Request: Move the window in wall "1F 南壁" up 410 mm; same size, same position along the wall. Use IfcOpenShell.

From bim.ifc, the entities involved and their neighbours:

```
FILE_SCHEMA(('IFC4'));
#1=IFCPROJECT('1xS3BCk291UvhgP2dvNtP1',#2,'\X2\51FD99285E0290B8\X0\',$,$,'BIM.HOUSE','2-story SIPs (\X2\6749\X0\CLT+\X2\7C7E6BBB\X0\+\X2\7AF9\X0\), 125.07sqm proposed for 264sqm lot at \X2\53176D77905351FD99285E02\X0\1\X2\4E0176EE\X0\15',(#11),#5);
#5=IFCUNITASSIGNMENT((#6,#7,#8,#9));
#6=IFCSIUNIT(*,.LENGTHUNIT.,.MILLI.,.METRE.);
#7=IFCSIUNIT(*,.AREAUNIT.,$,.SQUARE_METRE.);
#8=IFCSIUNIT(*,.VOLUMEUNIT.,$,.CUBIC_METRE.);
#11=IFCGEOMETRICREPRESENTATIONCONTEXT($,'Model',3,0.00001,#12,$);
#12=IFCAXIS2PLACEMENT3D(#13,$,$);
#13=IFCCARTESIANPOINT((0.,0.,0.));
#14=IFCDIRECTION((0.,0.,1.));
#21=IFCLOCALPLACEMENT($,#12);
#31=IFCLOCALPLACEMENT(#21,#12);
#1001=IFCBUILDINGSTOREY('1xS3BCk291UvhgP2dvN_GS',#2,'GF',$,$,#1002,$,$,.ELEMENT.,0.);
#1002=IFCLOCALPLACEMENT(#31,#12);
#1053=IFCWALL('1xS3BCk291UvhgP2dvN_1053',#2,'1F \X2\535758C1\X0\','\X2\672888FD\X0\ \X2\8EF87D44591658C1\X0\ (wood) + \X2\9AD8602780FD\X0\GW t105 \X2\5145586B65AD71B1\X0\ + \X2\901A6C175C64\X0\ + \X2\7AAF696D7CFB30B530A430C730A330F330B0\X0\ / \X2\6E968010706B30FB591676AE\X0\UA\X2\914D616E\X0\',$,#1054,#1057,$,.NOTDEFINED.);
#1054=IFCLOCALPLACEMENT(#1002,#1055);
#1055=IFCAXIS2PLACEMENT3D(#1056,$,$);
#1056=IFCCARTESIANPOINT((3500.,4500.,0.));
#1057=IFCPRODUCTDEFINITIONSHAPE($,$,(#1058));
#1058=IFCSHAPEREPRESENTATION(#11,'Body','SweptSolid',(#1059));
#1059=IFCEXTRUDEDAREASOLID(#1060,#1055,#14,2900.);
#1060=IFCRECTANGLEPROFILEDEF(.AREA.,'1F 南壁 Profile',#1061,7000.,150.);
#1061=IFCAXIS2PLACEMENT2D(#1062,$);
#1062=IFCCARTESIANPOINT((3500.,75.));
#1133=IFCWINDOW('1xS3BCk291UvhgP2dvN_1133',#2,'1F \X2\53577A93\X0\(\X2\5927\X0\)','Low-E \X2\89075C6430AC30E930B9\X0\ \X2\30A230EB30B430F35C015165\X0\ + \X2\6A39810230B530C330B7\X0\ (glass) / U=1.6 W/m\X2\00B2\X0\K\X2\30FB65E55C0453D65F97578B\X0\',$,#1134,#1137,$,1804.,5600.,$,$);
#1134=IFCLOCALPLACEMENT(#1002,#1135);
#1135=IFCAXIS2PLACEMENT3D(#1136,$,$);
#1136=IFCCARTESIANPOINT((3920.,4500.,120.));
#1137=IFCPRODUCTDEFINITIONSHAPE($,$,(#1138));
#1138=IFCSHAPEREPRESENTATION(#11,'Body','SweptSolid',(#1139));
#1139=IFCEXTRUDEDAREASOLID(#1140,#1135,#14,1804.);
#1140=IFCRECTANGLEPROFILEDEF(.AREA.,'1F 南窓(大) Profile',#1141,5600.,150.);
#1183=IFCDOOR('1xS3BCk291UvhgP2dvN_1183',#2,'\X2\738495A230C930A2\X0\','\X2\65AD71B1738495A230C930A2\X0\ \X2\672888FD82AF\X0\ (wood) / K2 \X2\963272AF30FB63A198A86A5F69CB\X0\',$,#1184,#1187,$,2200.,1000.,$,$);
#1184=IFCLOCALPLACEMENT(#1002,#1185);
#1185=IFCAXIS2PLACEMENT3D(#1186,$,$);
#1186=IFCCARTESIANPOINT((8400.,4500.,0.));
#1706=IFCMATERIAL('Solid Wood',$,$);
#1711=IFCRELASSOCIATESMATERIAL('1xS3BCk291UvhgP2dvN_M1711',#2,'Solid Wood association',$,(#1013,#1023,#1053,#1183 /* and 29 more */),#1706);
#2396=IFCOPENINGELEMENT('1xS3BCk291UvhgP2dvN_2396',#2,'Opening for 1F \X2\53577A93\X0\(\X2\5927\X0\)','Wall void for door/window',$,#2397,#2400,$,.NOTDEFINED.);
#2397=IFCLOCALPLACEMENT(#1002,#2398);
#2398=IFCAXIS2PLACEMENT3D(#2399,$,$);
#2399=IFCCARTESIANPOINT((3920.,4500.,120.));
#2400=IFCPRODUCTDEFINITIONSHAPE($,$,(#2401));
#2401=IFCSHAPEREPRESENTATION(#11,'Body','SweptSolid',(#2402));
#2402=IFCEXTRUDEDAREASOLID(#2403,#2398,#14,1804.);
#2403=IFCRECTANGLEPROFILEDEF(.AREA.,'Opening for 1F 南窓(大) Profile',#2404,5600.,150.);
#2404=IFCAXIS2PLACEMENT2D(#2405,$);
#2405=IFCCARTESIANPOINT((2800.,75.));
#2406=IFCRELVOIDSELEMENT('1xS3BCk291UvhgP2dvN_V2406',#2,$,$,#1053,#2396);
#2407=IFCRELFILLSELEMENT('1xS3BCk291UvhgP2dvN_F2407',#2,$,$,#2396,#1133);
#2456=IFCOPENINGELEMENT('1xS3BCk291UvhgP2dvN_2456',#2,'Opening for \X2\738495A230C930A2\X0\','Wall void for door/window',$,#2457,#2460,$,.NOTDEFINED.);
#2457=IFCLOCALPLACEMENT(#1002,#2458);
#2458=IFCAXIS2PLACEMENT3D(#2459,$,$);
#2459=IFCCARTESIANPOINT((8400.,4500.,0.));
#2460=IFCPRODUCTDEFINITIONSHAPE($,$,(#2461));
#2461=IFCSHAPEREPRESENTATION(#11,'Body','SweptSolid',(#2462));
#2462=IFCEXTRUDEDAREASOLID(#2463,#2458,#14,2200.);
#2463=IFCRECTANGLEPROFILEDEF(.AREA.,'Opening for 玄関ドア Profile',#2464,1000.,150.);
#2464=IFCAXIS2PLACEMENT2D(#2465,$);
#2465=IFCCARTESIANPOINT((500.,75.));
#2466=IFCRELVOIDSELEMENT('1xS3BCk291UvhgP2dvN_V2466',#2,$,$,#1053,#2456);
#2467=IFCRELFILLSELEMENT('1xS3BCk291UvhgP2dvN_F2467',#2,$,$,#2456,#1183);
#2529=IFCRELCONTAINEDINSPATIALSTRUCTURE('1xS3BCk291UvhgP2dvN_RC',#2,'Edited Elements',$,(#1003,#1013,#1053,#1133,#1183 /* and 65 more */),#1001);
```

```python
import numpy as np
import ifcopenshell
import ifcopenshell.api.geometry
import ifcopenshell.util.placement
import ifcopenshell.util.unit

model = ifcopenshell.open("bim.ifc")
unit_scale = ifcopenshell.util.unit.calculate_unit_scale(model)

window = model.by_guid("1xS3BCk291UvhgP2dvN_1133")
opening = window.FillsVoids[0].RelatingOpeningElement
dz = 0.41 / unit_scale

shift = np.array([0.0, 0.0, dz])
# The window is not placed relative to its opening, so move both.
for product in (opening, window):
    matrix = ifcopenshell.util.placement.get_local_placement(product.ObjectPlacement)
    matrix[:3, 3] += shift
    ifcopenshell.api.geometry.edit_object_placement(model, product=product, matrix=matrix, is_si=False)

print(f"moved by {dz * unit_scale:+.3f} m")

model.write("bim-out.ifc")
```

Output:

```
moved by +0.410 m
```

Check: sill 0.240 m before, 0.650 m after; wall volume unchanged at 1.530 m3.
